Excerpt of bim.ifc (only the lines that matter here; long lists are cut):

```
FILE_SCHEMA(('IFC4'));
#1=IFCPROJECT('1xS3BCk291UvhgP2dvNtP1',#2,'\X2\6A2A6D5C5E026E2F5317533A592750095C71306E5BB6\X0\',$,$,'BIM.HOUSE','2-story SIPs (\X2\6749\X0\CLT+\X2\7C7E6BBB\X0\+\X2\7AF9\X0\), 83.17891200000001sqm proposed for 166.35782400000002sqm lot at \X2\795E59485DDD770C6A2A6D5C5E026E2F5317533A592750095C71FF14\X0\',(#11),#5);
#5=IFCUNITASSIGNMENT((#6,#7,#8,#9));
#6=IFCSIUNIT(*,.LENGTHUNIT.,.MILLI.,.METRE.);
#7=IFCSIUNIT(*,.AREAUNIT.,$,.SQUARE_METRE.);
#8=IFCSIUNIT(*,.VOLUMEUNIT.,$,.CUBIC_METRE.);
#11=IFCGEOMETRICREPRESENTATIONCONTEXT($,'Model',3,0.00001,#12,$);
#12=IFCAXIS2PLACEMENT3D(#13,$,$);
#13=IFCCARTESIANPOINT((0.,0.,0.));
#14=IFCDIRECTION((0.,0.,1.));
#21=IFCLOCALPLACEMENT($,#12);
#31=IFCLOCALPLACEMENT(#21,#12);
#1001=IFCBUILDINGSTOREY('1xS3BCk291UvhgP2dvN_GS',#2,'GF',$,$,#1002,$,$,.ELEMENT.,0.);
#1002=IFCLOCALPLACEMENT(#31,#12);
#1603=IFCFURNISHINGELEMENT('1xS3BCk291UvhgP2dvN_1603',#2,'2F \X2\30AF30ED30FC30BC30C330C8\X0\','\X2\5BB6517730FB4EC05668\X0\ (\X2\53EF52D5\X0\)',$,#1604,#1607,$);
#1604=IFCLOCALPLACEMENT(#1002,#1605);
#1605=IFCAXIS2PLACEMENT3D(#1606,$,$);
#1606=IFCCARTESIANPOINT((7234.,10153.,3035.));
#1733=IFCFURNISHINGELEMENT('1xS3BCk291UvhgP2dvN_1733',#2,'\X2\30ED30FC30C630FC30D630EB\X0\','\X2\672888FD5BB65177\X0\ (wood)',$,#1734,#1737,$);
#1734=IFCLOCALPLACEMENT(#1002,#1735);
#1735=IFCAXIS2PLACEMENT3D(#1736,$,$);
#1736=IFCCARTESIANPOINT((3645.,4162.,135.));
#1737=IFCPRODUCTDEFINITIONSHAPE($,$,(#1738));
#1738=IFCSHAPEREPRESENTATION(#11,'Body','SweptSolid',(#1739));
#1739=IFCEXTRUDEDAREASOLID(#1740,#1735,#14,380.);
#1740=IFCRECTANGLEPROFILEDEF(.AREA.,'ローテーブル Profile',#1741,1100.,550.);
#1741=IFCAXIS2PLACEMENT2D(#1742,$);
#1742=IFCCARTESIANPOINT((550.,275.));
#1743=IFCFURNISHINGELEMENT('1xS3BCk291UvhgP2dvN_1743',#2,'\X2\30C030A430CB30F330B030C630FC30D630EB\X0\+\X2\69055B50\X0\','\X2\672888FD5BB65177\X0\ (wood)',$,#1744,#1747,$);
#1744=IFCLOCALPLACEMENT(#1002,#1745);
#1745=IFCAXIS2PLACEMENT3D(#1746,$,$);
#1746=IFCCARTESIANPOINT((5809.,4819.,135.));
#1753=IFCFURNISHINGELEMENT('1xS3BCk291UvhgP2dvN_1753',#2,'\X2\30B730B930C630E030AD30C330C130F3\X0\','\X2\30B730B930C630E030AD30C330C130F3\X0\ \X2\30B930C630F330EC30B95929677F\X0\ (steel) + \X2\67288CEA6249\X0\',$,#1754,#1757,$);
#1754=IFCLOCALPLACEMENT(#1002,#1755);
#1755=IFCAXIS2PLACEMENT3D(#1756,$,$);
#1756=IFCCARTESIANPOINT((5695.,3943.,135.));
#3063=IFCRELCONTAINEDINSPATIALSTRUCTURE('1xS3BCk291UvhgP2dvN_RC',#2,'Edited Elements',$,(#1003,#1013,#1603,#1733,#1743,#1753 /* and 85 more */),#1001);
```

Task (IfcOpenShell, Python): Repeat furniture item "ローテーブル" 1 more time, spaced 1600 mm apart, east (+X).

```python
import numpy as np
import ifcopenshell
import ifcopenshell.api.geometry
import ifcopenshell.api.root
import ifcopenshell.util.element
import ifcopenshell.util.placement
import ifcopenshell.util.unit

model = ifcopenshell.open("bim.ifc")
unit_scale = ifcopenshell.util.unit.calculate_unit_scale(model)


def reuse_history(source, copy):
    """copy_class also copies each property set's owner history, people and application; keep the originals."""
    for rel in copy.IsDefinedBy:
        if rel.is_a("IfcRelDefinesByProperties") and (history := rel.RelatingPropertyDefinition.OwnerHistory):
            rel.RelatingPropertyDefinition.OwnerHistory = source.OwnerHistory
            ifcopenshell.util.element.remove_deep2(model, history)


source = model.by_guid("1xS3BCk291UvhgP2dvN_1733")
base = ifcopenshell.util.placement.get_local_placement(source.ObjectPlacement)
step = np.array([1.0, 0.0, 0.0]) * 1.6 / unit_scale

for i in range(1, 2):
    copy = ifcopenshell.api.root.copy_class(model, product=source)
    copy.Representation = ifcopenshell.util.element.copy_deep(
        model, source.Representation, exclude=["IfcGeometricRepresentationContext", "IfcRepresentationMap"]
    )
    reuse_history(source, copy)
    matrix = base.copy()
    matrix[:3, 3] += i * step
    print("added at", matrix[:3, 3].round(3) + 0.0)
    ifcopenshell.api.geometry.edit_object_placement(model, product=copy, matrix=matrix, is_si=False)

model.write("bim_updated.ifc")
```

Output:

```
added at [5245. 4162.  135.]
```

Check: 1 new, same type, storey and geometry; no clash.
